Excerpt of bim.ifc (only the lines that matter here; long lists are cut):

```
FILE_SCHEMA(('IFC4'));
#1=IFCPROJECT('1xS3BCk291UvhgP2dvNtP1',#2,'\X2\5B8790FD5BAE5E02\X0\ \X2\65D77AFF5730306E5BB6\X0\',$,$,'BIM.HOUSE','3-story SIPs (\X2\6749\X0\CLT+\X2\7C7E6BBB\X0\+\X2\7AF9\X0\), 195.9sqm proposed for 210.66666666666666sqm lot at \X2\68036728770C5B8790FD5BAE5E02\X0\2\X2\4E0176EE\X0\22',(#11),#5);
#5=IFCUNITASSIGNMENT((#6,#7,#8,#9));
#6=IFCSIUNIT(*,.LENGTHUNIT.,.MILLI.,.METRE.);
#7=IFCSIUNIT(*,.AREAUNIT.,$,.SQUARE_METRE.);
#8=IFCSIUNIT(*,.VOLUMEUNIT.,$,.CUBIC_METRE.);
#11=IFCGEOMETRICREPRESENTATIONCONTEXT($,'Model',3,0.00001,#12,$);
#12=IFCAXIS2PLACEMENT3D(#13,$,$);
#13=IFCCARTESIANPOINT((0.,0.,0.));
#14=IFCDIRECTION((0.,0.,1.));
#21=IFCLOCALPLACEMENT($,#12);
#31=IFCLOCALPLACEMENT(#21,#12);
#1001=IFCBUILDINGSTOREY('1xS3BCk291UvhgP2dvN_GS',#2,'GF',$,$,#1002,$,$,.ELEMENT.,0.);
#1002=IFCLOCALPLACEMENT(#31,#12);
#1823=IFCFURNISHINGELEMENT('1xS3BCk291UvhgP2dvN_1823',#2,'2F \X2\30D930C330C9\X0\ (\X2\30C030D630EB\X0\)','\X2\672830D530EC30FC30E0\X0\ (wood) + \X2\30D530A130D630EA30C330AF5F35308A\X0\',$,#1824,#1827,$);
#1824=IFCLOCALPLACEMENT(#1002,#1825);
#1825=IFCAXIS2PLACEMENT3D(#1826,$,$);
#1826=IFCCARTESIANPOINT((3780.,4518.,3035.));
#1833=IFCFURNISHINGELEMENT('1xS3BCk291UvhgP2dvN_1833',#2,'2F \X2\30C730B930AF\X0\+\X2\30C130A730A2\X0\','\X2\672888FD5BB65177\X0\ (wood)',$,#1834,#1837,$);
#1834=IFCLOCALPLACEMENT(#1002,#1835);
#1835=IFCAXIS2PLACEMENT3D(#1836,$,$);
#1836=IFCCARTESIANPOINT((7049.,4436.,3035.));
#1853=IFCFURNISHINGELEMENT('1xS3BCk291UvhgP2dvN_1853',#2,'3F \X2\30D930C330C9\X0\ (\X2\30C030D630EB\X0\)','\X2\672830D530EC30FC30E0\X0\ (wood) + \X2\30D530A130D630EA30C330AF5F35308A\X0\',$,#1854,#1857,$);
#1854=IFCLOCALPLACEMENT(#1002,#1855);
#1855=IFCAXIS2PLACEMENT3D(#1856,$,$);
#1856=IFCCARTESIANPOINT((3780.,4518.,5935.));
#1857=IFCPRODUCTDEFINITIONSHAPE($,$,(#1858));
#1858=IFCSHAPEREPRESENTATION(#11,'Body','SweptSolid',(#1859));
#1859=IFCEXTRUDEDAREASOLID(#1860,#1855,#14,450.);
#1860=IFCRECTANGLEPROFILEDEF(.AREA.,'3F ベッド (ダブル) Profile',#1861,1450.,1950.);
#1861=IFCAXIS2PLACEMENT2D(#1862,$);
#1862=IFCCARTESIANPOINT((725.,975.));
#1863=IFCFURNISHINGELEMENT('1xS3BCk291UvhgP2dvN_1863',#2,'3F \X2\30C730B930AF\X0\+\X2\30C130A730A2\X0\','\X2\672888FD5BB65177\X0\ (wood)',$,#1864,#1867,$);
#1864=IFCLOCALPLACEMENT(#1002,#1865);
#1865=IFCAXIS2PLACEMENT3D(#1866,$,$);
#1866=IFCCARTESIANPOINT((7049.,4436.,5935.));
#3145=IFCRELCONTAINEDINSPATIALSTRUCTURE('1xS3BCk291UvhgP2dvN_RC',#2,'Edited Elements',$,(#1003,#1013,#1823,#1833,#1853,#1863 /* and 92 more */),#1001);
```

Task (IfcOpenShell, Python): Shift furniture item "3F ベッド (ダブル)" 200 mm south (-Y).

```python
import ifcopenshell
import ifcopenshell.api.geometry
import ifcopenshell.util.placement

model = ifcopenshell.open("bim.ifc")

item = model.by_id(1853)
matrix = ifcopenshell.util.placement.get_local_placement(item.ObjectPlacement)
matrix[1, 3] -= 200.0
ifcopenshell.api.geometry.edit_object_placement(model, product=item, matrix=matrix, is_si=False)

print(ifcopenshell.util.placement.get_local_placement(item.ObjectPlacement).round(3) + 0.0)

model.write("bim_updated.ifc")
```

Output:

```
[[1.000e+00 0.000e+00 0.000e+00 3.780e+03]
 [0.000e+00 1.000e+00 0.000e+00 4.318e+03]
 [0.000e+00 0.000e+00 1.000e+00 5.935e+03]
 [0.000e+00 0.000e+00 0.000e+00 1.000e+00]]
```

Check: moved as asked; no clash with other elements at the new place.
